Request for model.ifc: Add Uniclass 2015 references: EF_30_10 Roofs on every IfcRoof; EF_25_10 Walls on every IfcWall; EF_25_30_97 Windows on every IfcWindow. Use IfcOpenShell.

First a look at what the model holds.

```python
import ifcopenshell

model = ifcopenshell.open("model.ifc")
print(model.schema)
print("classifications:", [c.Name for c in model.by_type("IfcClassification")])
for ifc_class in ("IfcDoor", "IfcRoof", "IfcStair", "IfcWall", "IfcWindow"):
    print(ifc_class, len(model.by_type(ifc_class)))
```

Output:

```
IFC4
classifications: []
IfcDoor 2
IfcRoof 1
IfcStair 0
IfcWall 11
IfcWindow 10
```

```python
import ifcopenshell
import ifcopenshell.api.classification

model = ifcopenshell.open("model.ifc")

system = ifcopenshell.api.classification.add_classification(model, classification="Uniclass 2015")

codes = {
    "IfcRoof": ("EF_30_10", "Roofs"),
    "IfcWall": ("EF_25_10", "Walls"),
    "IfcWindow": ("EF_25_30_97", "Windows"),
}
for ifc_class, (code, name) in codes.items():
    products = model.by_type(ifc_class)
    ifcopenshell.api.classification.add_reference(
        model, products=products, classification=system, identification=code, name=name
    )
    print(code, len(products))

model.write("model-out.ifc")
```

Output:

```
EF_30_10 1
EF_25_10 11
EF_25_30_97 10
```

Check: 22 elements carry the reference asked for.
